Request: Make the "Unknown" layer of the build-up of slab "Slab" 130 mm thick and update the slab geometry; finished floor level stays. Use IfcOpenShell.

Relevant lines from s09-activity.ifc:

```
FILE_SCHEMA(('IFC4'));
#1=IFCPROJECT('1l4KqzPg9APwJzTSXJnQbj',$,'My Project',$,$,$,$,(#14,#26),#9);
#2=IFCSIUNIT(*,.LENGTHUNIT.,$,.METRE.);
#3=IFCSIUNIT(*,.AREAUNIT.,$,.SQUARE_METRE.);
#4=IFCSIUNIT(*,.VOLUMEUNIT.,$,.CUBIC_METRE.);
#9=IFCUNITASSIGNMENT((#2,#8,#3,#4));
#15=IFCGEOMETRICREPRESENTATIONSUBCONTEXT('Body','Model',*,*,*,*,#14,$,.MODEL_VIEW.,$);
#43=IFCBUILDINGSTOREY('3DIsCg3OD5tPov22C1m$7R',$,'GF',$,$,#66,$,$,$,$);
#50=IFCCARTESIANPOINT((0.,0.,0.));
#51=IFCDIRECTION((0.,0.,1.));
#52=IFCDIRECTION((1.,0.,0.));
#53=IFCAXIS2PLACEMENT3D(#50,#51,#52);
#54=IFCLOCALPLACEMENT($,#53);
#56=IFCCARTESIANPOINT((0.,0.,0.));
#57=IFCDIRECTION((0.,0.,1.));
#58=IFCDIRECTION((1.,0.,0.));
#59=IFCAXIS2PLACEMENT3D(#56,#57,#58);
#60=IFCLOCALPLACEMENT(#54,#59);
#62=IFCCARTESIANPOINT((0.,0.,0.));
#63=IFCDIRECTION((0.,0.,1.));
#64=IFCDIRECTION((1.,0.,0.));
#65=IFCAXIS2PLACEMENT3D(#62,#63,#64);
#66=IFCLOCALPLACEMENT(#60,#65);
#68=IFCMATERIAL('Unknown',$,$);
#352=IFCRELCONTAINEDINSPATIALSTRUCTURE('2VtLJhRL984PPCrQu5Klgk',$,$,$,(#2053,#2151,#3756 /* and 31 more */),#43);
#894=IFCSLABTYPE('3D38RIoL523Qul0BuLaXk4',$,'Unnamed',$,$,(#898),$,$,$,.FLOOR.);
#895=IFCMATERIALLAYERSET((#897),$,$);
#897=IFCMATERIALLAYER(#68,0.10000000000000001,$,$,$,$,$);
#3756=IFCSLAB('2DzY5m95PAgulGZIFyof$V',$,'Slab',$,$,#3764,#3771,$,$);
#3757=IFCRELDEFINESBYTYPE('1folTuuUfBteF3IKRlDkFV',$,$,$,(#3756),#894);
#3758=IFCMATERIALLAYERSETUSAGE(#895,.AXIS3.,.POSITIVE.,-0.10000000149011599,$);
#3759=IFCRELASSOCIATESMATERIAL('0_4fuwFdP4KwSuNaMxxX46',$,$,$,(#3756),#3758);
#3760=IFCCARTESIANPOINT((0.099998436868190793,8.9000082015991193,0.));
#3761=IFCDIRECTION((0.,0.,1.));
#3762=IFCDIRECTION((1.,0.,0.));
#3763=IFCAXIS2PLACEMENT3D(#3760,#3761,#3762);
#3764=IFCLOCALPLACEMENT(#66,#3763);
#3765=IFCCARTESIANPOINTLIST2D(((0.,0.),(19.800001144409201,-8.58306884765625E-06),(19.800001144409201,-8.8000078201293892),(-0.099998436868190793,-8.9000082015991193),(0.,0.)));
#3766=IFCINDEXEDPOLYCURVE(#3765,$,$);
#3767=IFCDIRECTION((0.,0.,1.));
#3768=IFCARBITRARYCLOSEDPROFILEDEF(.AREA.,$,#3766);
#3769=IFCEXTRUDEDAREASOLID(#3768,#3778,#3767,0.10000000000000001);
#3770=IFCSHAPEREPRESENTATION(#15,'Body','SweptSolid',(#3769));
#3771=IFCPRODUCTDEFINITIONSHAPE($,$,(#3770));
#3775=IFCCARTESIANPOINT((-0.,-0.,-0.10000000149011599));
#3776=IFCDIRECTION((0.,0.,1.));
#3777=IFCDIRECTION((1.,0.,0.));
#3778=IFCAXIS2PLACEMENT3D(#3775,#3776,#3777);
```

```python
import ifcopenshell
import ifcopenshell.util.element
import ifcopenshell.util.representation

model = ifcopenshell.open("s09-activity.ifc")

layer_set = model.by_id(895)
layer = next(l for l in layer_set.MaterialLayers if l.Material and l.Material.Name == "Unknown")
change = 0.13 - layer.LayerThickness
layer.LayerThickness += change

# Geometry does not follow the layer set by itself.
slabs = [e for e in ifcopenshell.util.element.get_elements_by_material(model, layer_set) if e.is_a("IfcSlab")]
for slab in sorted(slabs, key=lambda e: e.id()):
    body = ifcopenshell.util.representation.get_representation(slab, "Model", "Body")
    solid = body.Items[0]
    old_depth = solid.Depth
    solid.Depth += change
    # Extruded upwards: lower the start of the extrusion so the top stays.
    x, y, z = solid.Position.Location.Coordinates
    solid.Position.Location = model.createIfcCartesianPoint((x, y, z - change))
    print(slab.id(), f"{old_depth:g} -> {solid.Depth:g}")

# The layers are counted up from the underside, which has moved.
for usage in {ifcopenshell.util.element.get_material(slab) for slab in slabs}:
    usage.OffsetFromReferenceLine -= change

model.write("s09-activity_updated.ifc")
```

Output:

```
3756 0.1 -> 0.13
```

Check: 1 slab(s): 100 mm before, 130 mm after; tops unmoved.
